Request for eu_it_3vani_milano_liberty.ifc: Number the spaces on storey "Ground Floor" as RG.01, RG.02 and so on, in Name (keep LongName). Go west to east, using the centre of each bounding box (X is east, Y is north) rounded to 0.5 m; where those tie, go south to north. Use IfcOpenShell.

First a look at what the model holds.

```python
import ifcopenshell
import ifcopenshell.util.element
import ifcopenshell.util.placement

model = ifcopenshell.open("eu_it_3vani_milano_liberty.ifc")
print(model.schema)
storey = next(s for s in model.by_type("IfcBuildingStorey") if s.Name == "Ground Floor")
spaces = [e for e in ifcopenshell.util.element.get_decomposition(storey) if e.is_a("IfcSpace")]
for e in sorted(spaces, key=lambda e: e.id()):
    origin = ifcopenshell.util.placement.get_local_placement(e.ObjectPlacement)[:3, 3]
    print(e.id(), e.Name, e.LongName, origin.round(2) + 0.0, sep=" | ")
```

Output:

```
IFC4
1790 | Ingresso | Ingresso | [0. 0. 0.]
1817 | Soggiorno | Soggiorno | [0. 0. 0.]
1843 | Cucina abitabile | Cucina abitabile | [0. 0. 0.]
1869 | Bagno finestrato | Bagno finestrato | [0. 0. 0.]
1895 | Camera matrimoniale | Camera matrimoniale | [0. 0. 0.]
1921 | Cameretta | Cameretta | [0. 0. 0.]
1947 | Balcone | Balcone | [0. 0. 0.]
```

```python
import ifcopenshell
import ifcopenshell.geom
import ifcopenshell.util.element
import ifcopenshell.util.shape

model = ifcopenshell.open("eu_it_3vani_milano_liberty.ifc")
settings = ifcopenshell.geom.settings()
settings.set("use-world-coords", True)


def centre(element):
    shape = ifcopenshell.geom.create_shape(settings, element)
    return ifcopenshell.util.shape.get_bbox_centroid(shape.geometry)


storey = next(s for s in model.by_type("IfcBuildingStorey") if s.Name == "Ground Floor")
spaces = [e for e in ifcopenshell.util.element.get_decomposition(storey) if e.is_a("IfcSpace")]

# Insertion points can sit at a corner or the storey origin, so sort by the geometry (in metres).
centres = {e: centre(e) for e in spaces}
spaces.sort(key=lambda e: (round(centres[e][0] / 0.5), centres[e][1]))

for i, e in enumerate(spaces, start=1):
    number = f"RG.{i:02d}"
    e.Name = number
    print(e.id(), number)

model.write("eu_it_3vani_milano_liberty_updated.ifc")
```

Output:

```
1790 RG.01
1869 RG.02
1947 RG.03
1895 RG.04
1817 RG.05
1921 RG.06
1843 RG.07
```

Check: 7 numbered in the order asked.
